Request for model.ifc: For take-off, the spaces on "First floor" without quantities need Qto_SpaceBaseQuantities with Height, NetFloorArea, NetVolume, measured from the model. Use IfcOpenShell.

First a look at what the model holds.

```python
import ifcopenshell
import ifcopenshell.util.element
import ifcopenshell.util.unit

model = ifcopenshell.open("model.ifc")
print(model.schema)
for unit_type in ("LENGTHUNIT", "AREAUNIT", "VOLUMEUNIT"):
    print(unit_type, ifcopenshell.util.unit.calculate_unit_scale(model, unit_type))
storey = next(s for s in model.by_type("IfcBuildingStorey") if s.Name == "First floor")
spaces = [e for e in ifcopenshell.util.element.get_decomposition(storey) if e.is_a("IfcSpace")]
for e in sorted(spaces, key=lambda e: e.id()):
    print(e.id(), e.is_a(), e.Name, list(ifcopenshell.util.element.get_psets(e, qtos_only=True)), sep=" | ")
```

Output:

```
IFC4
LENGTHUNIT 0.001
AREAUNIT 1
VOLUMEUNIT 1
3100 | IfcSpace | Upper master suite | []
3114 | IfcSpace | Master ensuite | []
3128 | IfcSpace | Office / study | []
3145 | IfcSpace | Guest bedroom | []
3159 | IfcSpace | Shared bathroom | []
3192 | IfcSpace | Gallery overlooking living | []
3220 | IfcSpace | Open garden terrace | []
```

```python
import ifcopenshell
import ifcopenshell.api.pset
import ifcopenshell.geom
import ifcopenshell.util.element
import ifcopenshell.util.shape
import ifcopenshell.util.unit

model = ifcopenshell.open("model.ifc")
unit_scale = ifcopenshell.util.unit.calculate_unit_scale(model)
area_scale = ifcopenshell.util.unit.calculate_unit_scale(model, "AREAUNIT")
volume_scale = ifcopenshell.util.unit.calculate_unit_scale(model, "VOLUMEUNIT")
settings = ifcopenshell.geom.settings()

storey = next(s for s in model.by_type("IfcBuildingStorey") if s.Name == "First floor")
spaces = [e for e in ifcopenshell.util.element.get_decomposition(storey) if e.is_a("IfcSpace")]

for e in sorted(spaces, key=lambda e: e.id()):
    if ifcopenshell.util.element.get_psets(e, qtos_only=True, should_inherit=False):
        continue
    # Geometry comes back in metres, in the element's own axes.
    shape = ifcopenshell.geom.create_shape(settings, e)
    values = {
        "Height": ifcopenshell.util.shape.get_z(shape.geometry) / unit_scale,
        "NetFloorArea": ifcopenshell.util.shape.get_footprint_area(shape.geometry) / area_scale,
        "NetVolume": ifcopenshell.util.shape.get_volume(shape.geometry) / volume_scale,
    }
    qto = ifcopenshell.api.pset.add_qto(model, product=e, name="Qto_SpaceBaseQuantities")
    ifcopenshell.api.pset.edit_qto(model, qto=qto, properties=values)
    print(e.id(), {k: round(v, 3) for k, v in values.items()})

model.write("model_updated.ifc")
```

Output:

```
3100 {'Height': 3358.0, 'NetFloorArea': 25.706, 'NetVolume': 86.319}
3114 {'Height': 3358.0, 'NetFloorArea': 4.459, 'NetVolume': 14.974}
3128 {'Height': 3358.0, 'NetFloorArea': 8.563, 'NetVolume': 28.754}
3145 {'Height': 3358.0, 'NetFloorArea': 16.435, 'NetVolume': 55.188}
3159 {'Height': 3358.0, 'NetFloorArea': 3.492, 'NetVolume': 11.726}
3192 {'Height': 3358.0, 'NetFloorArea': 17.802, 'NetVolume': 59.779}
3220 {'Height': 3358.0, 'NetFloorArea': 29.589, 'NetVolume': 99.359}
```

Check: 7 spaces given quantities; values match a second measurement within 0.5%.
